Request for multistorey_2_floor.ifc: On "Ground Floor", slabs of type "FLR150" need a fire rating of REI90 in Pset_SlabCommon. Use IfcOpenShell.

First a look at what the model holds.

```python
import ifcopenshell
import ifcopenshell.util.element

model = ifcopenshell.open("multistorey_2_floor.ifc")
print(model.schema)
storey = next(s for s in model.by_type("IfcBuildingStorey") if s.Name == "Ground Floor")
slabs = [e for e in ifcopenshell.util.element.get_decomposition(storey) if e.is_a("IfcSlab")]
seen = {}
for e in slabs:
    element_type = ifcopenshell.util.element.get_type(e)
    key = (element_type.Name if element_type != e and element_type else None, ifcopenshell.util.element.get_pset(e, "Pset_SlabCommon", "FireRating"))
    seen[key] = seen.get(key, 0) + 1
for (name, value), count in sorted(seen.items(), key=str):
    print(count, "x", name, "|", value)
```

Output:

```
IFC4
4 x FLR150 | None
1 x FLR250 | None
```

```python
import ifcopenshell
import ifcopenshell.api.pset
import ifcopenshell.util.element

model = ifcopenshell.open("multistorey_2_floor.ifc")

storey = next(s for s in model.by_type("IfcBuildingStorey") if s.Name == "Ground Floor")
slabs = [e for e in ifcopenshell.util.element.get_decomposition(storey) if e.is_a("IfcSlab")]

count = 0
for e in slabs:
    element_type = ifcopenshell.util.element.get_type(e)
    if element_type in (None, e) or element_type.Name != "FLR150":
        continue
    # add_pset returns the element's existing set when there is one.
    pset = ifcopenshell.api.pset.add_pset(model, product=e, name="Pset_SlabCommon")
    ifcopenshell.api.pset.edit_pset(model, pset=pset, properties={"FireRating": "REI90"})
    count += 1

print(count, "slabs updated")

model.write("multistorey_2_floor_updated.ifc")
```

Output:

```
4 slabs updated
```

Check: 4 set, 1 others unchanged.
